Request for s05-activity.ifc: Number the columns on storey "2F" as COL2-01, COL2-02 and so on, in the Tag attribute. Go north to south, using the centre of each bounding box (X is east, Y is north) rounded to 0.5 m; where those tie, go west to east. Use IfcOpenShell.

First a look at what the model holds.

```python
import ifcopenshell
import ifcopenshell.util.element
import ifcopenshell.util.placement

model = ifcopenshell.open("s05-activity.ifc")
print(model.schema)
storey = next(s for s in model.by_type("IfcBuildingStorey") if s.Name == "2F")
columns = [e for e in ifcopenshell.util.element.get_decomposition(storey) if e.is_a("IfcColumn")]
for e in sorted(columns, key=lambda e: e.id()):
    origin = ifcopenshell.util.placement.get_local_placement(e.ObjectPlacement)[:3, 3]
    print(e.id(), e.Tag, e.Name, origin.round(2) + 0.0, sep=" | ")
```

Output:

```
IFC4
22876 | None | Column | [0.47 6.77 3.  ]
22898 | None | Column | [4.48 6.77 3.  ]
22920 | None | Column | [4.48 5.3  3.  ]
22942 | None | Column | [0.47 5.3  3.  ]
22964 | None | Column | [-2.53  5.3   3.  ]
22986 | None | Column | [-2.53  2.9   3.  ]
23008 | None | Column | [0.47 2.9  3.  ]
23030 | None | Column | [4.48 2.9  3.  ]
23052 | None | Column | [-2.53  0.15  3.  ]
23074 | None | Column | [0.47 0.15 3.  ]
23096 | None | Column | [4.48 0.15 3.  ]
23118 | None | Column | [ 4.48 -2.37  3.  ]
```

```python
import ifcopenshell
import ifcopenshell.geom
import ifcopenshell.util.element
import ifcopenshell.util.shape

model = ifcopenshell.open("s05-activity.ifc")
settings = ifcopenshell.geom.settings()
settings.set("use-world-coords", True)


def centre(element):
    shape = ifcopenshell.geom.create_shape(settings, element)
    return ifcopenshell.util.shape.get_bbox_centroid(shape.geometry)


storey = next(s for s in model.by_type("IfcBuildingStorey") if s.Name == "2F")
columns = [e for e in ifcopenshell.util.element.get_decomposition(storey) if e.is_a("IfcColumn")]

# Insertion points can sit at a corner or the storey origin, so sort by the geometry (in metres).
centres = {e: centre(e) for e in columns}
columns.sort(key=lambda e: (-round(centres[e][1] / 0.5), centres[e][0]))

for i, e in enumerate(columns, start=1):
    number = f"COL2-{i:02d}"
    e.Tag = number
    print(e.id(), number)

model.write("s05-activity_rev.ifc")
```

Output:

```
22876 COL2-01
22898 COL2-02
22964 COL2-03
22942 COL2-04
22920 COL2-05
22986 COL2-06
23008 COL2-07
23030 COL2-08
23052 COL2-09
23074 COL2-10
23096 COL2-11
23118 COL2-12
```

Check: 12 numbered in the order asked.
